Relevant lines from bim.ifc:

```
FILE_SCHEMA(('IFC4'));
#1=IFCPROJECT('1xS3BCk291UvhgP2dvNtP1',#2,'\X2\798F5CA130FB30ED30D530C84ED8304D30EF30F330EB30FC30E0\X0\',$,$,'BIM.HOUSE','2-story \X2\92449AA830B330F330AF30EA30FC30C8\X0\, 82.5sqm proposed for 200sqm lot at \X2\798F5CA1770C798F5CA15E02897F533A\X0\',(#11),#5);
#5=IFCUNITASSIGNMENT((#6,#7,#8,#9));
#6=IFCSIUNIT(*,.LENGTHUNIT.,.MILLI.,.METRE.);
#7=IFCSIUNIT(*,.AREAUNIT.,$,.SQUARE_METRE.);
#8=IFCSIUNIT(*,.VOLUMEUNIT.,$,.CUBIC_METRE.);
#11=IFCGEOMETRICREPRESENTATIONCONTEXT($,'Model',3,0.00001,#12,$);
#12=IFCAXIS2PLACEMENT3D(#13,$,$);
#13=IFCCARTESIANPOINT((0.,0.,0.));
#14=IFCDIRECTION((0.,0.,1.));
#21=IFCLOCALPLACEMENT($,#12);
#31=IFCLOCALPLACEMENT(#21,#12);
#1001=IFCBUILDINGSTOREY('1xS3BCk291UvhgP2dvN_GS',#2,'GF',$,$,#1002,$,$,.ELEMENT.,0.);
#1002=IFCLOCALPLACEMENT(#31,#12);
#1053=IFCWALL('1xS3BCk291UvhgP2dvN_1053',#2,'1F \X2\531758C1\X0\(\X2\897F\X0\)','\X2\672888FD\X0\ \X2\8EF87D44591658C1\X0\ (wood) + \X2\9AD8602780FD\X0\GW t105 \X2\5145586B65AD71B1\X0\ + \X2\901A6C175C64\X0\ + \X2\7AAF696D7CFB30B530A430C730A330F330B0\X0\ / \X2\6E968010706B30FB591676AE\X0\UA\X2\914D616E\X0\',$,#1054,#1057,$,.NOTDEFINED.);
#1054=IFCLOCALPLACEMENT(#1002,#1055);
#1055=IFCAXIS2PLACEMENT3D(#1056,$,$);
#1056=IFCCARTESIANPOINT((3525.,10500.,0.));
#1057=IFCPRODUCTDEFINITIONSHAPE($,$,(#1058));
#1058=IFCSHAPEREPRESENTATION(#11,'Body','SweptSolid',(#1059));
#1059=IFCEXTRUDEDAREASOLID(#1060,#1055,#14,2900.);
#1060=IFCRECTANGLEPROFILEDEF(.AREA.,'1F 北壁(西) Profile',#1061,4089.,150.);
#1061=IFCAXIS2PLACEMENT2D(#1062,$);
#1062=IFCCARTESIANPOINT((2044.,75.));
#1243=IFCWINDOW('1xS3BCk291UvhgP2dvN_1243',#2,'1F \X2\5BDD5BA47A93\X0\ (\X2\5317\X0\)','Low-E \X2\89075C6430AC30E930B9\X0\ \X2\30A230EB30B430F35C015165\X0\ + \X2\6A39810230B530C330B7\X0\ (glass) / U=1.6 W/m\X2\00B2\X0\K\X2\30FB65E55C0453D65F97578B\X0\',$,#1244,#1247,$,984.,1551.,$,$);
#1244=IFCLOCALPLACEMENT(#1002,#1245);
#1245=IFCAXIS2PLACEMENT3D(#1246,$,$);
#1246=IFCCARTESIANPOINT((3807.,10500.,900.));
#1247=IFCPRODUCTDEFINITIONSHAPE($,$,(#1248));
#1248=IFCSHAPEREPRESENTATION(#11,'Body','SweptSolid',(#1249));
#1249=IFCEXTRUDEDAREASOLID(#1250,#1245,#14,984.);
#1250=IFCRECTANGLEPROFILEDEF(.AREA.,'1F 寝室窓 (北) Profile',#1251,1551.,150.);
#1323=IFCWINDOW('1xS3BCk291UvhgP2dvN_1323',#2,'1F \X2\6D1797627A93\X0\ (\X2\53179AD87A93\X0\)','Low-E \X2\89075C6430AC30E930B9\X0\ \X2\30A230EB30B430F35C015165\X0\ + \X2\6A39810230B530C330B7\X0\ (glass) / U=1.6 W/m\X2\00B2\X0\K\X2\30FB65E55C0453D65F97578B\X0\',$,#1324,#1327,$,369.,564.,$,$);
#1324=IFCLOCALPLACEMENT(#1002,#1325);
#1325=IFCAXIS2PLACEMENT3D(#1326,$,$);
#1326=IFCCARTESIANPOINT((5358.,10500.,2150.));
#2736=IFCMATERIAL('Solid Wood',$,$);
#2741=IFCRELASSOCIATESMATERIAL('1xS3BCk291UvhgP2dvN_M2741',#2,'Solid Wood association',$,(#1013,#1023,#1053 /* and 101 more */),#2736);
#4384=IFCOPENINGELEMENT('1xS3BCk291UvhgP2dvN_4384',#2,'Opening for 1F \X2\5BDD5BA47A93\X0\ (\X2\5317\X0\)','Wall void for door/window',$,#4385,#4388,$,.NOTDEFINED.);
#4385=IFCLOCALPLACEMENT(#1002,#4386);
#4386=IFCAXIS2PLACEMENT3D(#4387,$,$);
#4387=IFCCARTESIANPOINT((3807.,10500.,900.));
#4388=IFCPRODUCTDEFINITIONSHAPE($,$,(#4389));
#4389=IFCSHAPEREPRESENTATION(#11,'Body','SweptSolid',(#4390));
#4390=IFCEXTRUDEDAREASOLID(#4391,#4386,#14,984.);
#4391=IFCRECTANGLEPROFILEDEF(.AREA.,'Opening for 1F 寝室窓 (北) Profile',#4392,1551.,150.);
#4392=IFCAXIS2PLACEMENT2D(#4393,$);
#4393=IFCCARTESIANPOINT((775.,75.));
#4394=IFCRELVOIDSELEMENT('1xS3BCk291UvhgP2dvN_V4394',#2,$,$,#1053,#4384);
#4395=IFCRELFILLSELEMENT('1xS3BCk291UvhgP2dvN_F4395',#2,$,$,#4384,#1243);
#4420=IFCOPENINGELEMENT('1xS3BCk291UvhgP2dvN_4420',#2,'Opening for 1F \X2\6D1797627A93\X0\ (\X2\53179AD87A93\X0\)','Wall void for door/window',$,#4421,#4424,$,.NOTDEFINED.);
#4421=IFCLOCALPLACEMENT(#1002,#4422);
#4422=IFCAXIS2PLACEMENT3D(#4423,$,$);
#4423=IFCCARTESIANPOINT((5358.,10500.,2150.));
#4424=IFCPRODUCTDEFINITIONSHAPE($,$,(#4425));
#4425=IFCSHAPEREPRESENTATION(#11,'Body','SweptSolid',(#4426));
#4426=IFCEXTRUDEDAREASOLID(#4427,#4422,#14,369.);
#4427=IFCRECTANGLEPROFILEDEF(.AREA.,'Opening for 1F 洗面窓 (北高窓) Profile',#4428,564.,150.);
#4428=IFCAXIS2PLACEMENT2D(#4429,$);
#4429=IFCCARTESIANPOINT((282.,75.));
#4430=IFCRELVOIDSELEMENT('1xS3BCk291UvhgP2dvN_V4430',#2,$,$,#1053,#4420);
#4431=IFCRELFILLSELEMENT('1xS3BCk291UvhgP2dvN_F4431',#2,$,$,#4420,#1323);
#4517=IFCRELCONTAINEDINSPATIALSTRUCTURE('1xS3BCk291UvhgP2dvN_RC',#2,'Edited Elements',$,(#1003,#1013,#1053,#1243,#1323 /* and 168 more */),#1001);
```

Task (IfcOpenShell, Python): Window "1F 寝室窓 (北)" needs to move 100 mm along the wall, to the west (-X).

```python
import ifcopenshell
import ifcopenshell.api.geometry
import ifcopenshell.util.placement
import ifcopenshell.util.unit

model = ifcopenshell.open("bim.ifc")
unit_scale = ifcopenshell.util.unit.calculate_unit_scale(model)

window = model.by_guid("1xS3BCk291UvhgP2dvN_1243")
opening = window.FillsVoids[0].RelatingOpeningElement
wall = opening.VoidsElements[0].RelatingBuildingElement

wall_matrix = ifcopenshell.util.placement.get_local_placement(wall.ObjectPlacement)
shift = wall_matrix[:3, 0] * -0.1 / unit_scale
before = ifcopenshell.util.placement.get_local_placement(window.ObjectPlacement)[:3, 3].copy()

# The window is not placed relative to its opening, so move both.
for product in (opening, window):
    matrix = ifcopenshell.util.placement.get_local_placement(product.ObjectPlacement)
    matrix[:3, 3] += shift
    ifcopenshell.api.geometry.edit_object_placement(model, product=product, matrix=matrix, is_si=False)

after = ifcopenshell.util.placement.get_local_placement(window.ObjectPlacement)[:3, 3]
print("window moved by", (after - before).round(3) + 0.0)

model.write("bim_rev.ifc")
```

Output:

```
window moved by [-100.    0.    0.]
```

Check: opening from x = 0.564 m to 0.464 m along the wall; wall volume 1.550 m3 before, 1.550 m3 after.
